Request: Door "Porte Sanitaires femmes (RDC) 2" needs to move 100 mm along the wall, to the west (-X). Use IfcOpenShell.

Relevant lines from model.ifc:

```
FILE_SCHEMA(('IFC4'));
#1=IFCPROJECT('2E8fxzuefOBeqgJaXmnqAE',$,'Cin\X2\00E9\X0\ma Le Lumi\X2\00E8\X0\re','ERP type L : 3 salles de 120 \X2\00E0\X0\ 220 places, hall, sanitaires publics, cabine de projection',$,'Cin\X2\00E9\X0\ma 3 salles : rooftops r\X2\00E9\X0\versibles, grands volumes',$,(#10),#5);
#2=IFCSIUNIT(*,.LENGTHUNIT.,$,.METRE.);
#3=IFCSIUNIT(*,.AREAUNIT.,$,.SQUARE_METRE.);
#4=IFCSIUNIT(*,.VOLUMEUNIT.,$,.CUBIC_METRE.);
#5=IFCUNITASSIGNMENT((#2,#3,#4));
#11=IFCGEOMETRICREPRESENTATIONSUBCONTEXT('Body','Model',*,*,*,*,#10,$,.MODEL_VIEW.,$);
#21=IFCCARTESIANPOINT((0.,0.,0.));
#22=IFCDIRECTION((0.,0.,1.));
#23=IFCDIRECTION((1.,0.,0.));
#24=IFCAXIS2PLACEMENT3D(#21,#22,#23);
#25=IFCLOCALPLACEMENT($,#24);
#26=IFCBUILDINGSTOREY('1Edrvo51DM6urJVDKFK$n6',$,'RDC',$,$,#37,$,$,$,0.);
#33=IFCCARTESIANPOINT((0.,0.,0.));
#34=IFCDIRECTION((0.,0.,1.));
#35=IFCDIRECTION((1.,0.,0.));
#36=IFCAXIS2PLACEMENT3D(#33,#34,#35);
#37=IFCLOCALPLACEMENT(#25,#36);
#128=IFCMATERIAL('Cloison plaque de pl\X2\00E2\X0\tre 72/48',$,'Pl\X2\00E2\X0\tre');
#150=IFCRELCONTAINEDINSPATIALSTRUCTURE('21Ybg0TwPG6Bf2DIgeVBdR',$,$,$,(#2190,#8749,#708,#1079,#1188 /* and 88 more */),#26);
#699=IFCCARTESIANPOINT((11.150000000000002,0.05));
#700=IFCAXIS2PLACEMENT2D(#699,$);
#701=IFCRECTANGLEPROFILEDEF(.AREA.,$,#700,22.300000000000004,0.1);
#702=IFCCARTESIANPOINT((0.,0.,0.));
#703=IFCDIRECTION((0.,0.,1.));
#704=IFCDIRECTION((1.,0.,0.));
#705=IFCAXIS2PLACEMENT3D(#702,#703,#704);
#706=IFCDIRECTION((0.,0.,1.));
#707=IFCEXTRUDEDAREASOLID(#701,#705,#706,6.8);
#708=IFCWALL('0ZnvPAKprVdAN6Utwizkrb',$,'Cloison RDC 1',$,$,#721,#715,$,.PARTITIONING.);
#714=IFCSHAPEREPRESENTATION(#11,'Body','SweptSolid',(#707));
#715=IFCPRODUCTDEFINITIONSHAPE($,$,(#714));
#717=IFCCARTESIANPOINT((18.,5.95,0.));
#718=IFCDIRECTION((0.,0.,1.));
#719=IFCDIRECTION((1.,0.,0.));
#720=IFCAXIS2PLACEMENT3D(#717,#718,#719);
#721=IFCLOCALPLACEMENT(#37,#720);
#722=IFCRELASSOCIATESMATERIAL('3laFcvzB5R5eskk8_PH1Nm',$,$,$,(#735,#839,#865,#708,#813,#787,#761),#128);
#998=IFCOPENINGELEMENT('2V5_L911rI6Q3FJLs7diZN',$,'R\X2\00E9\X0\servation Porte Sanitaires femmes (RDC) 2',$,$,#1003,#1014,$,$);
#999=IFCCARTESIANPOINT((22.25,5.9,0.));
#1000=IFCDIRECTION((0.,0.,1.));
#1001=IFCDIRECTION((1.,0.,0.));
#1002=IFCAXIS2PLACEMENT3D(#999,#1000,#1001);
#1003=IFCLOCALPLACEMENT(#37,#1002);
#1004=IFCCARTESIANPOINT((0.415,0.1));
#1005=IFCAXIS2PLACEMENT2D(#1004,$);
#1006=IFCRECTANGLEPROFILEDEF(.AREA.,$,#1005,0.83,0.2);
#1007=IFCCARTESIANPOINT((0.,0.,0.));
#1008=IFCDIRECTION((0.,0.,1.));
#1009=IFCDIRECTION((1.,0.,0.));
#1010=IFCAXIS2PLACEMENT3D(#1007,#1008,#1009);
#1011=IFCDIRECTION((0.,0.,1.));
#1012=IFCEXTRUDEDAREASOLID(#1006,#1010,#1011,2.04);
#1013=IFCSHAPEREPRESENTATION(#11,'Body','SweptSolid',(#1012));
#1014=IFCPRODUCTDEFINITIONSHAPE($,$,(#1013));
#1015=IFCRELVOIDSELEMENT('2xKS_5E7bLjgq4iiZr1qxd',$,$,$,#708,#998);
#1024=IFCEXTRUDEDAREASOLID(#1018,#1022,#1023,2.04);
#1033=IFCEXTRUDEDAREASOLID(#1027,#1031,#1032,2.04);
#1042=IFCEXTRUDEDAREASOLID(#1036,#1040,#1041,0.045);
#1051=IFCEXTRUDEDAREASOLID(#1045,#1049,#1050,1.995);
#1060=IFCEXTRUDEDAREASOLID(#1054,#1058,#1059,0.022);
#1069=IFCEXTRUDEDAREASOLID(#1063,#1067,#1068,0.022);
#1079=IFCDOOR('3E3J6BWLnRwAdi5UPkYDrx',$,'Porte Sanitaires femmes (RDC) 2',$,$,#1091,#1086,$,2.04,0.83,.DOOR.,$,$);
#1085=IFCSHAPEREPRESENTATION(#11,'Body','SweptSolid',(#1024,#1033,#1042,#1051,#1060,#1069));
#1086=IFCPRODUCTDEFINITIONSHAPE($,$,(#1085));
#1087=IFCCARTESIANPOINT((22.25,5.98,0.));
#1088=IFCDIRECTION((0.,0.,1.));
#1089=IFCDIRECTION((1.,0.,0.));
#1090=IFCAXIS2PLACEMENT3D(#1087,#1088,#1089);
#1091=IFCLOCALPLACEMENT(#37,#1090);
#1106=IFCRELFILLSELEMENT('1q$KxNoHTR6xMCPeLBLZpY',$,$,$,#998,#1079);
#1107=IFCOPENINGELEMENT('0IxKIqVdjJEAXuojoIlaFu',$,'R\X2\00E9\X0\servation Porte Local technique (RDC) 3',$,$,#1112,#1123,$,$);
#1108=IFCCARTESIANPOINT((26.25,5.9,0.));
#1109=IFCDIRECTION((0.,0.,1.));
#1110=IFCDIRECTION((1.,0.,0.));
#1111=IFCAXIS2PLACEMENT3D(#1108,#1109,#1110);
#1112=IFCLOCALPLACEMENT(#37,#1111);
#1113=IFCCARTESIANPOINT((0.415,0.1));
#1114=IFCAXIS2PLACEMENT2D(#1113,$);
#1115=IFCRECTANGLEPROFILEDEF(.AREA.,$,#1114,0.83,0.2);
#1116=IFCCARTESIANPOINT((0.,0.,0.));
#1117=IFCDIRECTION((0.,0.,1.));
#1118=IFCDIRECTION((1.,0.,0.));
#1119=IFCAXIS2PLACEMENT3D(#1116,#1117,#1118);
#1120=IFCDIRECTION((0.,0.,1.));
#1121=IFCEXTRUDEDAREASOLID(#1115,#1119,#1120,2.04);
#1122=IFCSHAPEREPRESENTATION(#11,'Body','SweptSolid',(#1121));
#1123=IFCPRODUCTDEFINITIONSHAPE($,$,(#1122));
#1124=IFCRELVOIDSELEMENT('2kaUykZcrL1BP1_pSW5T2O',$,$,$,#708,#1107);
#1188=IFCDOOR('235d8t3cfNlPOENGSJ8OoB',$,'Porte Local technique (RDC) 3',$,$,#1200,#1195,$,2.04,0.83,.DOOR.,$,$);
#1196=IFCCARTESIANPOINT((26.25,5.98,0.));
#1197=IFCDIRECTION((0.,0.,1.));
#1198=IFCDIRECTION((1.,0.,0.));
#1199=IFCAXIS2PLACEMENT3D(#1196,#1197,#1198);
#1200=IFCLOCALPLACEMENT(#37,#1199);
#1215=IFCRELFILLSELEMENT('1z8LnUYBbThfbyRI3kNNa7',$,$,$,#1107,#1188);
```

```python
import ifcopenshell
import ifcopenshell.api.geometry
import ifcopenshell.util.placement
import ifcopenshell.util.unit

model = ifcopenshell.open("model.ifc")
unit_scale = ifcopenshell.util.unit.calculate_unit_scale(model)

door = model.by_guid("3E3J6BWLnRwAdi5UPkYDrx")
opening = door.FillsVoids[0].RelatingOpeningElement
wall = opening.VoidsElements[0].RelatingBuildingElement

wall_matrix = ifcopenshell.util.placement.get_local_placement(wall.ObjectPlacement)
shift = wall_matrix[:3, 0] * -0.1 / unit_scale
before = ifcopenshell.util.placement.get_local_placement(door.ObjectPlacement)[:3, 3].copy()

# The door is not placed relative to its opening, so move both.
for product in (opening, door):
    matrix = ifcopenshell.util.placement.get_local_placement(product.ObjectPlacement)
    matrix[:3, 3] += shift
    ifcopenshell.api.geometry.edit_object_placement(model, product=product, matrix=matrix, is_si=False)

after = ifcopenshell.util.placement.get_local_placement(door.ObjectPlacement)[:3, 3]
print("door moved by", (after - before).round(3) + 0.0)

model.write("model_edited.ifc")
```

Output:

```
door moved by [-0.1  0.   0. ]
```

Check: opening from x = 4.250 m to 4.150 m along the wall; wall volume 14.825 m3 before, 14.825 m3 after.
